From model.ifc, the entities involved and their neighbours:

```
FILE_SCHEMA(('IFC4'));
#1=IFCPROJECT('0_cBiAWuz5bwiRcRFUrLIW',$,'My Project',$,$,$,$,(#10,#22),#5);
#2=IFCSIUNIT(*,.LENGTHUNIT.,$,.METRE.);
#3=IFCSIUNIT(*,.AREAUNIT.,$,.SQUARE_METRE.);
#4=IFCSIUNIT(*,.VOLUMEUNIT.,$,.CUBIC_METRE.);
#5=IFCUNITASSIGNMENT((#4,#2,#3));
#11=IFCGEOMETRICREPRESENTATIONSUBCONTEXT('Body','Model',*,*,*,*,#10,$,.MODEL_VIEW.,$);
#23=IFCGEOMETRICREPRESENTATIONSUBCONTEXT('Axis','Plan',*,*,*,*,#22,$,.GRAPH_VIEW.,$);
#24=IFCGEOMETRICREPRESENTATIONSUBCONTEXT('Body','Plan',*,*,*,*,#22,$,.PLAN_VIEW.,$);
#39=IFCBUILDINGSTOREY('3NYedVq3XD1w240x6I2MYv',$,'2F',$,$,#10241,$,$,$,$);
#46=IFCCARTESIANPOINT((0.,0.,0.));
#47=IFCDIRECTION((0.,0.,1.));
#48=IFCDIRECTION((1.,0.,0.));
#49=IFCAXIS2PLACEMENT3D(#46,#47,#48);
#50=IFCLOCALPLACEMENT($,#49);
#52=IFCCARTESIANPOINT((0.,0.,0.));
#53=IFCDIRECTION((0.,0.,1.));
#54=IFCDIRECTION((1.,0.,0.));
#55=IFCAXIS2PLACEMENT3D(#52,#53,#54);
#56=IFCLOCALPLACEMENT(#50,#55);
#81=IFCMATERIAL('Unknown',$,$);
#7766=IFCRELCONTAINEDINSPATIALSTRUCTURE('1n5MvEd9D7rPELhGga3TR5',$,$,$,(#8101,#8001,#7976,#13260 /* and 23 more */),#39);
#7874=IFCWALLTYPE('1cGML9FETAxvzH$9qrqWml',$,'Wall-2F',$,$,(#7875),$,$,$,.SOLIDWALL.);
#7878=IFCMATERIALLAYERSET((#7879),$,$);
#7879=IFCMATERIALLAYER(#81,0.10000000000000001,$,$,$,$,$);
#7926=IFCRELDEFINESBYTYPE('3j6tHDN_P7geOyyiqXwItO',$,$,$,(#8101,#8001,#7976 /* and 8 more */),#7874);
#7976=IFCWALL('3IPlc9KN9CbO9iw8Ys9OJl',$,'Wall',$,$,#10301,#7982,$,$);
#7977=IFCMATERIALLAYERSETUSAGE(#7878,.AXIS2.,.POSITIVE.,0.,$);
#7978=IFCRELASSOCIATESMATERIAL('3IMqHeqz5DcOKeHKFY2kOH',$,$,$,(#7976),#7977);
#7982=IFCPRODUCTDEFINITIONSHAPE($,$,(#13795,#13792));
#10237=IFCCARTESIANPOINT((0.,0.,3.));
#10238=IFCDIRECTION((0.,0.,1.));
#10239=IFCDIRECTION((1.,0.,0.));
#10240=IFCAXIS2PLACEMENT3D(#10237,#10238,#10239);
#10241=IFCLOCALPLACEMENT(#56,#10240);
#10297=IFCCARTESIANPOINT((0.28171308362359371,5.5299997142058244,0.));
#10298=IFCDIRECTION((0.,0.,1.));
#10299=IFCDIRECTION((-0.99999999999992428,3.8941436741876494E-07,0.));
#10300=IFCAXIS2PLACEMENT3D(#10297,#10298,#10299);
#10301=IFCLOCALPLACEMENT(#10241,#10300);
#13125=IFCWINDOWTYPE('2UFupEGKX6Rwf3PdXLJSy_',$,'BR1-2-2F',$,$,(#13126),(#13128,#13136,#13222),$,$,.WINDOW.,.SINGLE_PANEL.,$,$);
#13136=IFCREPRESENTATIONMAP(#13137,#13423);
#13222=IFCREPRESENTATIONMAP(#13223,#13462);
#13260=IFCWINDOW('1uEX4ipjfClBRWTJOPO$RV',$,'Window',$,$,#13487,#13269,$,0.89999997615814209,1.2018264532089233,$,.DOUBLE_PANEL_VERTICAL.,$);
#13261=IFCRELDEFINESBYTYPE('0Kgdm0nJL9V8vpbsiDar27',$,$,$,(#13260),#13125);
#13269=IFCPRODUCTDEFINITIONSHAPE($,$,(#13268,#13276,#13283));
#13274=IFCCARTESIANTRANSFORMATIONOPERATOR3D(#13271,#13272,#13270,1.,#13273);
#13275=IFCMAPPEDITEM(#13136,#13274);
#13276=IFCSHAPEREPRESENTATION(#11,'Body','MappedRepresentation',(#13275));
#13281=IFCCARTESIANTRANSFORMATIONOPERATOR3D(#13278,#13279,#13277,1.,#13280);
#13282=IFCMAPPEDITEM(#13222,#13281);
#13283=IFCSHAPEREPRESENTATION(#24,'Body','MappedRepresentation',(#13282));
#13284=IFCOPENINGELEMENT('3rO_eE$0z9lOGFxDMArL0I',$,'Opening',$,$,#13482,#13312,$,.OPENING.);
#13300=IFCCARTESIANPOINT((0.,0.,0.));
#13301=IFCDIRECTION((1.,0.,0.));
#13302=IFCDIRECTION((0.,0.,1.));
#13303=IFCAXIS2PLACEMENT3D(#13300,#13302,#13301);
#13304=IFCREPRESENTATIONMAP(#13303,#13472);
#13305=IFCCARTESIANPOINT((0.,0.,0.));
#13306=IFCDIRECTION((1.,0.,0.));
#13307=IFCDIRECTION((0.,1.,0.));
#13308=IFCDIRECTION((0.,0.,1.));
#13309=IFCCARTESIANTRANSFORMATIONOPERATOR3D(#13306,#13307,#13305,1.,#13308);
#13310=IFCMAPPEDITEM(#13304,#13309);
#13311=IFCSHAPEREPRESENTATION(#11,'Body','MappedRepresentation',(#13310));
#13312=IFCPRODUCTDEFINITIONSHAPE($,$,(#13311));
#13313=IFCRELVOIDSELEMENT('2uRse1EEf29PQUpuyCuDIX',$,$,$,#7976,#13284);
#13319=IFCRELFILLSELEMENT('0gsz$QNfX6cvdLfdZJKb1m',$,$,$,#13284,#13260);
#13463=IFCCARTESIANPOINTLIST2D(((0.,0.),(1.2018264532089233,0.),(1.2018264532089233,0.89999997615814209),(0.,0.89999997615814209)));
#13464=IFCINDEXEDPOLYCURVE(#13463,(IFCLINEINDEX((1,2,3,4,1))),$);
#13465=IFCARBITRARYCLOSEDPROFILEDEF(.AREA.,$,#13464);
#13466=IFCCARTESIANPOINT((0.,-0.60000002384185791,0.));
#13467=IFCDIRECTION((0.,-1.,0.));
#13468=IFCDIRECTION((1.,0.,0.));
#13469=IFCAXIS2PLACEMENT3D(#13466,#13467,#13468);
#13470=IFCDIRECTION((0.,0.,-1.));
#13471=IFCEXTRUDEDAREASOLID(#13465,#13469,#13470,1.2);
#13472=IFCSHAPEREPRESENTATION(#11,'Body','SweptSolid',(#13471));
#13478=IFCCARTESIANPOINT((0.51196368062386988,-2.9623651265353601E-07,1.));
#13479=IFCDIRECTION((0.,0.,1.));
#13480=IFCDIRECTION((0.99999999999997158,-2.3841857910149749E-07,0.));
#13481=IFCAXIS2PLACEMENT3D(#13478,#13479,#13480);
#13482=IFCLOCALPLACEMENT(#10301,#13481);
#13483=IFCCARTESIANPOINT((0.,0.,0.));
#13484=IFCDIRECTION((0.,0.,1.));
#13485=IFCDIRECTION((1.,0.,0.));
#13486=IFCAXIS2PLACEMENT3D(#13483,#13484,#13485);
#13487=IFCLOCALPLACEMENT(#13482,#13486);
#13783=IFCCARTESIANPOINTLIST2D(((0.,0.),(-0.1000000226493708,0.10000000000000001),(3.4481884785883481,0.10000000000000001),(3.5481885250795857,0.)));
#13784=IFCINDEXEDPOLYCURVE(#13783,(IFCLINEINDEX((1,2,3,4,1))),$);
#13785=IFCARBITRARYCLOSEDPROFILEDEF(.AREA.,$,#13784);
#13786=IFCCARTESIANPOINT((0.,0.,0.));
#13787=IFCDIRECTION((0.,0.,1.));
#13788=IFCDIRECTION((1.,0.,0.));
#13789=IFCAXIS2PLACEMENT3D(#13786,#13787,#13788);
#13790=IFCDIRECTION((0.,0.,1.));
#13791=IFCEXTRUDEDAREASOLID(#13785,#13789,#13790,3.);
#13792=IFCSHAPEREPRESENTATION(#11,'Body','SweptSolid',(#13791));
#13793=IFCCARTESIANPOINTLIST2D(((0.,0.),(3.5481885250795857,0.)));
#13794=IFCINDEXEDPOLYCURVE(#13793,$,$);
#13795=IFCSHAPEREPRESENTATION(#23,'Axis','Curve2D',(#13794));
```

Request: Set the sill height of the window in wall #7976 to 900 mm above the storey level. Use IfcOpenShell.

```python
import numpy as np
import ifcopenshell
import ifcopenshell.api.geometry
import ifcopenshell.geom
import ifcopenshell.util.element
import ifcopenshell.util.placement
import ifcopenshell.util.shape
import ifcopenshell.util.unit

model = ifcopenshell.open("model.ifc")
unit_scale = ifcopenshell.util.unit.calculate_unit_scale(model)

window = model.by_id(13260)
opening = window.FillsVoids[0].RelatingOpeningElement
storey = ifcopenshell.util.element.get_container(window, ifc_class="IfcBuildingStorey")
level = ifcopenshell.util.placement.get_local_placement(storey.ObjectPlacement)[2, 3]

# The opening's origin need not be at the sill, so measure its lowest point.
shape = ifcopenshell.geom.create_shape(ifcopenshell.geom.settings(), opening)
bottom = ifcopenshell.util.shape.get_shape_bottom_elevation(shape, shape.geometry) / unit_scale
dz = level + 0.9 / unit_scale - bottom

shift = np.array([0.0, 0.0, dz])
# The window is placed relative to its opening, so it follows when the opening moves.
matrix = ifcopenshell.util.placement.get_local_placement(opening.ObjectPlacement)
matrix[:3, 3] += shift
ifcopenshell.api.geometry.edit_object_placement(
    model, product=opening, matrix=matrix, is_si=False, should_transform_children=True
)

print(f"moved by {dz * unit_scale:+.3f} m")

model.write("model_updated.ifc")
```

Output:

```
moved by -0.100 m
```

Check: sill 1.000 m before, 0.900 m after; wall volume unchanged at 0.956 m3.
